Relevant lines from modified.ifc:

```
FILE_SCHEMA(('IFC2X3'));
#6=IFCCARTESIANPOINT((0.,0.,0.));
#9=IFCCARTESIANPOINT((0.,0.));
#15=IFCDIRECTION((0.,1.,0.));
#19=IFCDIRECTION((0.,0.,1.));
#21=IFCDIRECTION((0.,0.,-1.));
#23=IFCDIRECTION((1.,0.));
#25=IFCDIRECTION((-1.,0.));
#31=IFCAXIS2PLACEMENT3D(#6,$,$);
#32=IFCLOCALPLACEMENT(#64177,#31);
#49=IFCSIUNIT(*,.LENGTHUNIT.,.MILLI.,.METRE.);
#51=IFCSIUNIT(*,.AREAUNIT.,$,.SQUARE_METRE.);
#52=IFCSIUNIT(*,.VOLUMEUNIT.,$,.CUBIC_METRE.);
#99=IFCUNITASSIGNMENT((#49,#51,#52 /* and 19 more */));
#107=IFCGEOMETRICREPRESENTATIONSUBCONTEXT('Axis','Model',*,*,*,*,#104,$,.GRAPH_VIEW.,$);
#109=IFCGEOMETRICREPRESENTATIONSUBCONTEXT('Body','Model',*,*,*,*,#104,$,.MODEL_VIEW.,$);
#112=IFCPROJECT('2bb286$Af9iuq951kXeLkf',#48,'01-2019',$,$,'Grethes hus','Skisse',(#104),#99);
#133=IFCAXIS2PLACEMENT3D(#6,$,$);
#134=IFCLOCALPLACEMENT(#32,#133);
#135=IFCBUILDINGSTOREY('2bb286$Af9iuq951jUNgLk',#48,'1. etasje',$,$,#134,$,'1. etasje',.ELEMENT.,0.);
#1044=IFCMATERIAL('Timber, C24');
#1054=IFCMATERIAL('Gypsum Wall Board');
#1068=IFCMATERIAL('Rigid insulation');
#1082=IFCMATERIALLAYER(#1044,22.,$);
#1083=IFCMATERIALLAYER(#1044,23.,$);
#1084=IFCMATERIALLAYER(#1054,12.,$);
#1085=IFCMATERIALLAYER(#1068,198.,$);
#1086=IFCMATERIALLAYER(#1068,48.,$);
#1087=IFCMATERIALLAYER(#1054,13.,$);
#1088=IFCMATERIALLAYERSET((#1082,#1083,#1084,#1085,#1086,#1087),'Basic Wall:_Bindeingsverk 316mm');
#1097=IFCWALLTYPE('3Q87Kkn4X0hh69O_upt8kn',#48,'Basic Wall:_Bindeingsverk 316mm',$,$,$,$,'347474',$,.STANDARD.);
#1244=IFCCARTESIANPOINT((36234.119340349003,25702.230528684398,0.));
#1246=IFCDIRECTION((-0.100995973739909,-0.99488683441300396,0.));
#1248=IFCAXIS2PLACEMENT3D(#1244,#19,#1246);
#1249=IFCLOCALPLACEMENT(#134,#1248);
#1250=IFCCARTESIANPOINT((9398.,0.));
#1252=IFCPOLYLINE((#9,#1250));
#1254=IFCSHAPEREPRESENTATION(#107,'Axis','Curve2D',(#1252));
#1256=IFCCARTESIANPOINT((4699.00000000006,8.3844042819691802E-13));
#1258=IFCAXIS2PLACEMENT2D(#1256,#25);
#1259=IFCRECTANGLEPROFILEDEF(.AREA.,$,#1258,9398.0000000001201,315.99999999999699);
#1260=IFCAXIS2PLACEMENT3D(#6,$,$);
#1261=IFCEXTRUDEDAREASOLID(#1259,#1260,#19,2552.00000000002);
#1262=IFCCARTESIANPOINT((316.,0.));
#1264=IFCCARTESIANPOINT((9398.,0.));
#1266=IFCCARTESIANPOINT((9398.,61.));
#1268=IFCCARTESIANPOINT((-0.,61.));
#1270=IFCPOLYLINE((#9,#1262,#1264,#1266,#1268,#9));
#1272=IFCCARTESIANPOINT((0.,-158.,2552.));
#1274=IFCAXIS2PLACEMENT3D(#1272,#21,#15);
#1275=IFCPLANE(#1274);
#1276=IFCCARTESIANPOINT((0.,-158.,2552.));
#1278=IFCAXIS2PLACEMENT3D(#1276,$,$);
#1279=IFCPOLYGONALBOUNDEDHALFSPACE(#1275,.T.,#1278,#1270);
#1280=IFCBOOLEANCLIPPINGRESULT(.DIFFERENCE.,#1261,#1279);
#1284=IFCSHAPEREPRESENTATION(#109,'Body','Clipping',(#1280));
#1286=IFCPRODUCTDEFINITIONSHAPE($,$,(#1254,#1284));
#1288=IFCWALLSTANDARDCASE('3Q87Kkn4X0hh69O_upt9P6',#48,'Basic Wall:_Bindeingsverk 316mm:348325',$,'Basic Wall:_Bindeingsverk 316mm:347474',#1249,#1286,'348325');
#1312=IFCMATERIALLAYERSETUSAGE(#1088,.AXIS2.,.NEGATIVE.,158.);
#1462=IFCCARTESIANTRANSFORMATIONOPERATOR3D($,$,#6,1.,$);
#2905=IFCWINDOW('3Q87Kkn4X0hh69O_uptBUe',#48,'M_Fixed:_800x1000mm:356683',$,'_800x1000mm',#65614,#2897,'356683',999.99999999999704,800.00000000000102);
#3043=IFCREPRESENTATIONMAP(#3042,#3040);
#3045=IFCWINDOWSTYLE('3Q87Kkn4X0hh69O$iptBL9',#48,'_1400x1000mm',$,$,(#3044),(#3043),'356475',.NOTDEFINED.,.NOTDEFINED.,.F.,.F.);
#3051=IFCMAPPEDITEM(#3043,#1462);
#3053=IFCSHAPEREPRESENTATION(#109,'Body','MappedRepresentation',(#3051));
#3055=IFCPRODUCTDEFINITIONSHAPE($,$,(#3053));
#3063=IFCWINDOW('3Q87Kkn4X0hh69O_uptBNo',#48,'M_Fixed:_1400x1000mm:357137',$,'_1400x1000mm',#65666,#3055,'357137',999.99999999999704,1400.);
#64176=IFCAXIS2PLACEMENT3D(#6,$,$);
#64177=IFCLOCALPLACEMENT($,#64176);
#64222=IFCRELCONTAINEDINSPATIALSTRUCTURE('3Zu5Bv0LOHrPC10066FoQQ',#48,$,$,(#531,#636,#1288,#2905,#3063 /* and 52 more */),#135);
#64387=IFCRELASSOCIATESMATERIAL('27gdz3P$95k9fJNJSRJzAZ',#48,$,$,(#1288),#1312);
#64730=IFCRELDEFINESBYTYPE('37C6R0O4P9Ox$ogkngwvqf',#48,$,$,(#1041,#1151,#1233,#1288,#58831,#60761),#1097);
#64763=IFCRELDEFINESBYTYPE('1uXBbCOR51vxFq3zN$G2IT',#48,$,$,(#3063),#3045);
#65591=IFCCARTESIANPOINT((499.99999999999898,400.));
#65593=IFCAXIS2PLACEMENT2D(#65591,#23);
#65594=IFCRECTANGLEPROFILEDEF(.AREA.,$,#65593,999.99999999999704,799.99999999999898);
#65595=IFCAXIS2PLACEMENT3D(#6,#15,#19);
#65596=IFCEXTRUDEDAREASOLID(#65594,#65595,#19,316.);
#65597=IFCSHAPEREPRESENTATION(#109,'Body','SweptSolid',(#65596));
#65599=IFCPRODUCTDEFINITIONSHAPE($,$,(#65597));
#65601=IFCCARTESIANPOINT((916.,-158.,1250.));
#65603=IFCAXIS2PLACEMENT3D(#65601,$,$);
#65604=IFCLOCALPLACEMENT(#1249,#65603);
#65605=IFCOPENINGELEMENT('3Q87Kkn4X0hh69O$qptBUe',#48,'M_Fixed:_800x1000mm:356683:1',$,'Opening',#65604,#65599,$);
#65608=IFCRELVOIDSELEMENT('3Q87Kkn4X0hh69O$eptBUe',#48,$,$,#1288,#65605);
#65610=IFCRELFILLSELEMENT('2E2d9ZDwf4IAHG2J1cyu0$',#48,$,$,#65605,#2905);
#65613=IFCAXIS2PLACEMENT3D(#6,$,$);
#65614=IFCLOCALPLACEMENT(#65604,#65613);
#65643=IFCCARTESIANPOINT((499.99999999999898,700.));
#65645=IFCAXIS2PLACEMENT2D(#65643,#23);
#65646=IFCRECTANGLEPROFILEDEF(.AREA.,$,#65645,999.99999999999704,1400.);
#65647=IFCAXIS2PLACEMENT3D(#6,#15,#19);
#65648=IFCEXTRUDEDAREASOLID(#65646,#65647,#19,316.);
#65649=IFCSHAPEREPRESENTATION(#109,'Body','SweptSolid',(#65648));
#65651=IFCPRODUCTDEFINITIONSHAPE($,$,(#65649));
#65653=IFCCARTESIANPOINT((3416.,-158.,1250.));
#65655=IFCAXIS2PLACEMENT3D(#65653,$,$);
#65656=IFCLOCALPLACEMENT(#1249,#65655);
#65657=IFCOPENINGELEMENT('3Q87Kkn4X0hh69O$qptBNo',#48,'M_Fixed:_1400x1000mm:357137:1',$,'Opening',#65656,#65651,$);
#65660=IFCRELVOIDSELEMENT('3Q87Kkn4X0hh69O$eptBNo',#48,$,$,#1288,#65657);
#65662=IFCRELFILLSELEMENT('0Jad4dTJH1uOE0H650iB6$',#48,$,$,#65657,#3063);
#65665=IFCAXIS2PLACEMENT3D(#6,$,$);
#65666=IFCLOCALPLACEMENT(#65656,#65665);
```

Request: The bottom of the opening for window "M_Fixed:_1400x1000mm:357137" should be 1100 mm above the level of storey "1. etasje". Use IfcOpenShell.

```python
import numpy as np
import ifcopenshell
import ifcopenshell.api.geometry
import ifcopenshell.geom
import ifcopenshell.util.element
import ifcopenshell.util.placement
import ifcopenshell.util.shape
import ifcopenshell.util.unit

model = ifcopenshell.open("modified.ifc")
unit_scale = ifcopenshell.util.unit.calculate_unit_scale(model)

window = model.by_guid("3Q87Kkn4X0hh69O_uptBNo")
opening = window.FillsVoids[0].RelatingOpeningElement
storey = ifcopenshell.util.element.get_container(window, ifc_class="IfcBuildingStorey")
level = ifcopenshell.util.placement.get_local_placement(storey.ObjectPlacement)[2, 3]

# The opening's origin need not be at the sill, so measure its lowest point.
shape = ifcopenshell.geom.create_shape(ifcopenshell.geom.settings(), opening)
bottom = ifcopenshell.util.shape.get_shape_bottom_elevation(shape, shape.geometry) / unit_scale
dz = level + 1.1 / unit_scale - bottom

shift = np.array([0.0, 0.0, dz])
# The window is placed relative to its opening, so it follows when the opening moves.
matrix = ifcopenshell.util.placement.get_local_placement(opening.ObjectPlacement)
matrix[:3, 3] += shift
ifcopenshell.api.geometry.edit_object_placement(
    model, product=opening, matrix=matrix, is_si=False, should_transform_children=True
)

print(f"moved by {dz * unit_scale:+.3f} m")

model.write("modified_edited.ifc")
```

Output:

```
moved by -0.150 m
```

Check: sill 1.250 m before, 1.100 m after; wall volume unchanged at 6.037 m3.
